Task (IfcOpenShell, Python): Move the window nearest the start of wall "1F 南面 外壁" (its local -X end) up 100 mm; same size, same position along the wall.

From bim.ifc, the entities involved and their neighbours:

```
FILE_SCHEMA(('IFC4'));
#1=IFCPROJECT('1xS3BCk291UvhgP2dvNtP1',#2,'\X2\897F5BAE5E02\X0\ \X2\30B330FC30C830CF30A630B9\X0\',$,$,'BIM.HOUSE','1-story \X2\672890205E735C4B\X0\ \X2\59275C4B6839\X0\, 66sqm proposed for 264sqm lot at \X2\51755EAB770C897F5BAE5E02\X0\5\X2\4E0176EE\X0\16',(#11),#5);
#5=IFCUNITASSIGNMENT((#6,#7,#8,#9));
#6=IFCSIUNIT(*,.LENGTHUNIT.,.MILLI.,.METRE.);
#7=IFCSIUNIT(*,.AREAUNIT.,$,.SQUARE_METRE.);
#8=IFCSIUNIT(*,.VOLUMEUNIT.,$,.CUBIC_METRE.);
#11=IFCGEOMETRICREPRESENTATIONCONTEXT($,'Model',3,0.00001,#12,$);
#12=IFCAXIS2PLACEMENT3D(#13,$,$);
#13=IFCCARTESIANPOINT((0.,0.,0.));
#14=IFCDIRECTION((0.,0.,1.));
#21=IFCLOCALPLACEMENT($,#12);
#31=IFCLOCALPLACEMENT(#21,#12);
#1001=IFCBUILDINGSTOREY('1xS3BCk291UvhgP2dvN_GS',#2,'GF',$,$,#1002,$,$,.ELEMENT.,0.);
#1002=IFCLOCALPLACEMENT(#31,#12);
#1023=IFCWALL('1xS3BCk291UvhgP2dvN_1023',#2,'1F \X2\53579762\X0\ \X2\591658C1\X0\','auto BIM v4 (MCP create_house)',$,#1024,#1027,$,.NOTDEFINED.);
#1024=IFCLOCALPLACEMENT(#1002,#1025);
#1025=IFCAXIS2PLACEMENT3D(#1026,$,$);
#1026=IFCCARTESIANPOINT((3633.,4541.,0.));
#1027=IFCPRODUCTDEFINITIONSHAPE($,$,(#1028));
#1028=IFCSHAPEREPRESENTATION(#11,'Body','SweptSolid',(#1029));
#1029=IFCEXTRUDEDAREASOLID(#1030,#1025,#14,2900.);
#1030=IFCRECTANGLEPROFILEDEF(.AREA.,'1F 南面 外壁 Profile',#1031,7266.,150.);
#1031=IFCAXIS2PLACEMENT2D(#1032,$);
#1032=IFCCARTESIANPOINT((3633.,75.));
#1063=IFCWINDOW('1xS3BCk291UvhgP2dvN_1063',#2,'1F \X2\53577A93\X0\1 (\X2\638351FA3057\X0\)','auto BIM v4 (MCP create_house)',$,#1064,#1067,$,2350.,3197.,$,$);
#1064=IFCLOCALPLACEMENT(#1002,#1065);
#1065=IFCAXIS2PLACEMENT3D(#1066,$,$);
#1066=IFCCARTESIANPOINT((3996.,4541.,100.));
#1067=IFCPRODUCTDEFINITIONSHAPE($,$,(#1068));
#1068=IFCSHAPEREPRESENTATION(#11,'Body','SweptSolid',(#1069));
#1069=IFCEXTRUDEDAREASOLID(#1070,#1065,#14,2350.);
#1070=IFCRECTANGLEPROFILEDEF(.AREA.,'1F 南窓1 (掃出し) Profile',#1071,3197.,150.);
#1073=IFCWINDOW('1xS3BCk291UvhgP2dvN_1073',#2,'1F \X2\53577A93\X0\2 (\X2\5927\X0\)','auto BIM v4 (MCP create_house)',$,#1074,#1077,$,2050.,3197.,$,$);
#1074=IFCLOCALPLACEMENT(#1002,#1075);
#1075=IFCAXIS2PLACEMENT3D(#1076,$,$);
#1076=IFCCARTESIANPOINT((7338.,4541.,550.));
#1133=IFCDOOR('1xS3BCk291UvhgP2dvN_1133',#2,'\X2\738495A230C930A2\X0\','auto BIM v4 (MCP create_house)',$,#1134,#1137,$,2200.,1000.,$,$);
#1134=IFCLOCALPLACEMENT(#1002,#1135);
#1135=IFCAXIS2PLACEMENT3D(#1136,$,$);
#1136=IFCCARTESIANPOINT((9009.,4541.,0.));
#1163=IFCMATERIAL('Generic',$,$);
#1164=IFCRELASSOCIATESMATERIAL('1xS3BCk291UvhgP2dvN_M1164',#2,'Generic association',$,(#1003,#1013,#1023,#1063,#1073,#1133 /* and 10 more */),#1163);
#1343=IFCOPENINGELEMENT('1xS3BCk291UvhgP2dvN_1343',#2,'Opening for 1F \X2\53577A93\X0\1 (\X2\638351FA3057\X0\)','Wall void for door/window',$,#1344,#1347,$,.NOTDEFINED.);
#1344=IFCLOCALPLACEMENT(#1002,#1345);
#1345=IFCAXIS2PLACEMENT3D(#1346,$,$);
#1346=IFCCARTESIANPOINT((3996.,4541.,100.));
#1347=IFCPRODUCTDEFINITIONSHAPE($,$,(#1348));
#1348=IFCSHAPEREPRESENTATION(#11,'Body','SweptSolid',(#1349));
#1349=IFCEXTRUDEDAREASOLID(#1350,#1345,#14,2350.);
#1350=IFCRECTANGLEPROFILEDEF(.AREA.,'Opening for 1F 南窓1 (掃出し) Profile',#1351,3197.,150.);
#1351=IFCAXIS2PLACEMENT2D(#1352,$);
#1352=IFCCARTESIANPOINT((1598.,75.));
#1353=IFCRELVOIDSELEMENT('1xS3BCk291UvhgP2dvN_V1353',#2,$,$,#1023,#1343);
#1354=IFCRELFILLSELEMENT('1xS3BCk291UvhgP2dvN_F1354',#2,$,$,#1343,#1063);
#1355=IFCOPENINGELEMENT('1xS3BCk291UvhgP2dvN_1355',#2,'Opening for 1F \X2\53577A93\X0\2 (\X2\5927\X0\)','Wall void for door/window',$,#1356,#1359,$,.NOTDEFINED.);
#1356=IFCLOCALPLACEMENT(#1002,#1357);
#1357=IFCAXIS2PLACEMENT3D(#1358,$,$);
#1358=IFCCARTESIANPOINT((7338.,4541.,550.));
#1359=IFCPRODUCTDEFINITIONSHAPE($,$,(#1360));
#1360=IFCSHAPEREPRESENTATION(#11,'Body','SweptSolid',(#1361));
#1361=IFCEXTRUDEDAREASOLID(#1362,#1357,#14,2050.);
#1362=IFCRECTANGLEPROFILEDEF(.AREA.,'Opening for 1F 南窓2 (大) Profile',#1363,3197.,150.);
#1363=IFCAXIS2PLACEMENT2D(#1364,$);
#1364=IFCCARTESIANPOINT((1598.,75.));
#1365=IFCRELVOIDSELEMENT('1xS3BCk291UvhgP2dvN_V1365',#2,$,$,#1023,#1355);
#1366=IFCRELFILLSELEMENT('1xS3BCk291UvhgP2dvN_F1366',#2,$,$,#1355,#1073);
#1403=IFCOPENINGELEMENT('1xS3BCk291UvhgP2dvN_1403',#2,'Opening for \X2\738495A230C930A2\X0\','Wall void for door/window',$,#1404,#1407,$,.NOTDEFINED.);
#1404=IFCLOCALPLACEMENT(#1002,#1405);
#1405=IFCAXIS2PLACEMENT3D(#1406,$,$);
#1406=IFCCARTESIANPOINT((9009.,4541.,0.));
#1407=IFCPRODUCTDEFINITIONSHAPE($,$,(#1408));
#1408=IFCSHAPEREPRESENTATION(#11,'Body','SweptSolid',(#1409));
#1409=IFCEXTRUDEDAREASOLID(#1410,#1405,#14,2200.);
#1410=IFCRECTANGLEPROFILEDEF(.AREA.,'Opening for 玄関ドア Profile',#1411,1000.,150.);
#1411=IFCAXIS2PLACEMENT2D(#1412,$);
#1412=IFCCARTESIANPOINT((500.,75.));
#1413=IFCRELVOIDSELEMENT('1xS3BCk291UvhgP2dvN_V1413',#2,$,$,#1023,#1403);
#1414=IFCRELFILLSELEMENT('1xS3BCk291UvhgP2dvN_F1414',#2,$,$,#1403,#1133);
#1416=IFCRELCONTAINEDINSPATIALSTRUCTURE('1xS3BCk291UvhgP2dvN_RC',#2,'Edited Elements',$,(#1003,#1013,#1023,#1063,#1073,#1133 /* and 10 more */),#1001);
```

```python
import numpy as np
import ifcopenshell
import ifcopenshell.api.geometry
import ifcopenshell.util.placement
import ifcopenshell.util.unit

model = ifcopenshell.open("bim.ifc")
unit_scale = ifcopenshell.util.unit.calculate_unit_scale(model)

window = model.by_id(1063)
opening = window.FillsVoids[0].RelatingOpeningElement
dz = 0.1 / unit_scale

shift = np.array([0.0, 0.0, dz])
# The window is not placed relative to its opening, so move both.
for product in (opening, window):
    matrix = ifcopenshell.util.placement.get_local_placement(product.ObjectPlacement)
    matrix[:3, 3] += shift
    ifcopenshell.api.geometry.edit_object_placement(model, product=product, matrix=matrix, is_si=False)

print(f"moved by {dz * unit_scale:+.3f} m")

model.write("bim_v2.ifc")
```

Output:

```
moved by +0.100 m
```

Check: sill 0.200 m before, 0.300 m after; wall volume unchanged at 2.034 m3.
